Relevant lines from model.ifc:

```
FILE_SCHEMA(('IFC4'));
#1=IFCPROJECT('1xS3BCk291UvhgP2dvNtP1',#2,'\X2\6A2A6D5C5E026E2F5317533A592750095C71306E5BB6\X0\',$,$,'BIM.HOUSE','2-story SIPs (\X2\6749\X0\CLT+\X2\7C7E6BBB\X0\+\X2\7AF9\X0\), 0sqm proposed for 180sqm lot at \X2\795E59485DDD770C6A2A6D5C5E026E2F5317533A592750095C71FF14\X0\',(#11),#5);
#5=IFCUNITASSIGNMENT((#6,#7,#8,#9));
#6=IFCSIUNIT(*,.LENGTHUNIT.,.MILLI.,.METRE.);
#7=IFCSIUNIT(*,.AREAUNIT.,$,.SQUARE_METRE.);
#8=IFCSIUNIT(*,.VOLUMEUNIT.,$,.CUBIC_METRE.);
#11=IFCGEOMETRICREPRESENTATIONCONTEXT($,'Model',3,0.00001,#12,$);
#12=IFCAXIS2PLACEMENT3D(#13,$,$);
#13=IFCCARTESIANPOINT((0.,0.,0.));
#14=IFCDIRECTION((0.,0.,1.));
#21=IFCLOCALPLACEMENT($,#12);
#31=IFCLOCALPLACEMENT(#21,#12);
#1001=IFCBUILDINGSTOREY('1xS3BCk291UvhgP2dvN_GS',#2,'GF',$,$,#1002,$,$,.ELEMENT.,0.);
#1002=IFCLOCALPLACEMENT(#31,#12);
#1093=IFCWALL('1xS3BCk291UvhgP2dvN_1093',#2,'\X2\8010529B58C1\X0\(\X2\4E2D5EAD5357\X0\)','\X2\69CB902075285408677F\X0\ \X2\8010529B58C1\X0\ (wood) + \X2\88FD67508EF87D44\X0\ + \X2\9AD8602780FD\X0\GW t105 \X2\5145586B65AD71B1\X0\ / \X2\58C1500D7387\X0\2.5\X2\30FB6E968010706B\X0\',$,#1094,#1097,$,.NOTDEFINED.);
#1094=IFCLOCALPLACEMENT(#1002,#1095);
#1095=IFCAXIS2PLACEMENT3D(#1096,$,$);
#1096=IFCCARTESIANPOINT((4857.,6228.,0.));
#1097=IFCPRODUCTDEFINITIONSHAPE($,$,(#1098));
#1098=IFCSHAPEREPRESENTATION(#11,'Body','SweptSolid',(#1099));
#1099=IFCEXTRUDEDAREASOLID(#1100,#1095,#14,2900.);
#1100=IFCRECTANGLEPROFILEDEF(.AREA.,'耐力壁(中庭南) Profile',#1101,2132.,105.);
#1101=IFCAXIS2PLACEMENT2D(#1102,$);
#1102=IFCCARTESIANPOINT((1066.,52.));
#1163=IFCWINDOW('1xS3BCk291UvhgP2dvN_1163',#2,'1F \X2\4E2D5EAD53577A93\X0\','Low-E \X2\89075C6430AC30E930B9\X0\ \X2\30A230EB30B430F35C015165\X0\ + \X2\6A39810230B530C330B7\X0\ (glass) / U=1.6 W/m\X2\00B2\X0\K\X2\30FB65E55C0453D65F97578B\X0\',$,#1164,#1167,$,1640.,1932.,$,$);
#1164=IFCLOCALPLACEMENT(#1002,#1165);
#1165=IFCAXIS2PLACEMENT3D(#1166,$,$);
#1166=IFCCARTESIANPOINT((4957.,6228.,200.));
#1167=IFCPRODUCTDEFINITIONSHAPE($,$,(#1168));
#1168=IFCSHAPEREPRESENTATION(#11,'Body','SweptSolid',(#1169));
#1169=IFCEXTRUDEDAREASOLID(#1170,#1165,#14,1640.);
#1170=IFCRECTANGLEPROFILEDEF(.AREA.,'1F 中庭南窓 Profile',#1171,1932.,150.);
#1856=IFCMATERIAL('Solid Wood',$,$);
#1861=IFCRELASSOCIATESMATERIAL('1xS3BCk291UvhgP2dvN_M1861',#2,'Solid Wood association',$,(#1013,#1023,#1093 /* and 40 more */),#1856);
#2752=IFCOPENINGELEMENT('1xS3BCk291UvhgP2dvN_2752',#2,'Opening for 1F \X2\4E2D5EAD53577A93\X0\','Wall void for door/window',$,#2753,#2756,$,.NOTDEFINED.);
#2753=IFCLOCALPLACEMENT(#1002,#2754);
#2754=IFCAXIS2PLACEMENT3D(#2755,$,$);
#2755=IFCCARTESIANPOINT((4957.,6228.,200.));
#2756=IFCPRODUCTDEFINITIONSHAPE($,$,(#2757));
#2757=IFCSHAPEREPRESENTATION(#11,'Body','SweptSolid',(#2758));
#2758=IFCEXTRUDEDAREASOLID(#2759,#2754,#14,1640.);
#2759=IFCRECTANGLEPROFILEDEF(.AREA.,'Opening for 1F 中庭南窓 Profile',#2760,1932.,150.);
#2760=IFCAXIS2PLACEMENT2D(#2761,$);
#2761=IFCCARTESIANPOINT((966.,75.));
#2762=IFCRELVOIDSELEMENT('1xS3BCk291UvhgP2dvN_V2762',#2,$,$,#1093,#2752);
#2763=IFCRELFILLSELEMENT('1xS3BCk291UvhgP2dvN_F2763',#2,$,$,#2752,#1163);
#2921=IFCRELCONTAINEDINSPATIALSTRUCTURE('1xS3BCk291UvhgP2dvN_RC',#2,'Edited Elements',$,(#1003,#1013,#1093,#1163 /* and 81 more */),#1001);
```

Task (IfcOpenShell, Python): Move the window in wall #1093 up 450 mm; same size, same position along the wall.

```python
import numpy as np
import ifcopenshell
import ifcopenshell.api.geometry
import ifcopenshell.util.placement
import ifcopenshell.util.unit

model = ifcopenshell.open("model.ifc")
unit_scale = ifcopenshell.util.unit.calculate_unit_scale(model)

window = model.by_guid("1xS3BCk291UvhgP2dvN_1163")
opening = window.FillsVoids[0].RelatingOpeningElement
dz = 0.45 / unit_scale

shift = np.array([0.0, 0.0, dz])
# The window is not placed relative to its opening, so move both.
for product in (opening, window):
    matrix = ifcopenshell.util.placement.get_local_placement(product.ObjectPlacement)
    matrix[:3, 3] += shift
    ifcopenshell.api.geometry.edit_object_placement(model, product=product, matrix=matrix, is_si=False)

print(f"moved by {dz * unit_scale:+.3f} m")

model.write("model_edited.ifc")
```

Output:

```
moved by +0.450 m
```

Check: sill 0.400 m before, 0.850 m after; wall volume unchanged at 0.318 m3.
